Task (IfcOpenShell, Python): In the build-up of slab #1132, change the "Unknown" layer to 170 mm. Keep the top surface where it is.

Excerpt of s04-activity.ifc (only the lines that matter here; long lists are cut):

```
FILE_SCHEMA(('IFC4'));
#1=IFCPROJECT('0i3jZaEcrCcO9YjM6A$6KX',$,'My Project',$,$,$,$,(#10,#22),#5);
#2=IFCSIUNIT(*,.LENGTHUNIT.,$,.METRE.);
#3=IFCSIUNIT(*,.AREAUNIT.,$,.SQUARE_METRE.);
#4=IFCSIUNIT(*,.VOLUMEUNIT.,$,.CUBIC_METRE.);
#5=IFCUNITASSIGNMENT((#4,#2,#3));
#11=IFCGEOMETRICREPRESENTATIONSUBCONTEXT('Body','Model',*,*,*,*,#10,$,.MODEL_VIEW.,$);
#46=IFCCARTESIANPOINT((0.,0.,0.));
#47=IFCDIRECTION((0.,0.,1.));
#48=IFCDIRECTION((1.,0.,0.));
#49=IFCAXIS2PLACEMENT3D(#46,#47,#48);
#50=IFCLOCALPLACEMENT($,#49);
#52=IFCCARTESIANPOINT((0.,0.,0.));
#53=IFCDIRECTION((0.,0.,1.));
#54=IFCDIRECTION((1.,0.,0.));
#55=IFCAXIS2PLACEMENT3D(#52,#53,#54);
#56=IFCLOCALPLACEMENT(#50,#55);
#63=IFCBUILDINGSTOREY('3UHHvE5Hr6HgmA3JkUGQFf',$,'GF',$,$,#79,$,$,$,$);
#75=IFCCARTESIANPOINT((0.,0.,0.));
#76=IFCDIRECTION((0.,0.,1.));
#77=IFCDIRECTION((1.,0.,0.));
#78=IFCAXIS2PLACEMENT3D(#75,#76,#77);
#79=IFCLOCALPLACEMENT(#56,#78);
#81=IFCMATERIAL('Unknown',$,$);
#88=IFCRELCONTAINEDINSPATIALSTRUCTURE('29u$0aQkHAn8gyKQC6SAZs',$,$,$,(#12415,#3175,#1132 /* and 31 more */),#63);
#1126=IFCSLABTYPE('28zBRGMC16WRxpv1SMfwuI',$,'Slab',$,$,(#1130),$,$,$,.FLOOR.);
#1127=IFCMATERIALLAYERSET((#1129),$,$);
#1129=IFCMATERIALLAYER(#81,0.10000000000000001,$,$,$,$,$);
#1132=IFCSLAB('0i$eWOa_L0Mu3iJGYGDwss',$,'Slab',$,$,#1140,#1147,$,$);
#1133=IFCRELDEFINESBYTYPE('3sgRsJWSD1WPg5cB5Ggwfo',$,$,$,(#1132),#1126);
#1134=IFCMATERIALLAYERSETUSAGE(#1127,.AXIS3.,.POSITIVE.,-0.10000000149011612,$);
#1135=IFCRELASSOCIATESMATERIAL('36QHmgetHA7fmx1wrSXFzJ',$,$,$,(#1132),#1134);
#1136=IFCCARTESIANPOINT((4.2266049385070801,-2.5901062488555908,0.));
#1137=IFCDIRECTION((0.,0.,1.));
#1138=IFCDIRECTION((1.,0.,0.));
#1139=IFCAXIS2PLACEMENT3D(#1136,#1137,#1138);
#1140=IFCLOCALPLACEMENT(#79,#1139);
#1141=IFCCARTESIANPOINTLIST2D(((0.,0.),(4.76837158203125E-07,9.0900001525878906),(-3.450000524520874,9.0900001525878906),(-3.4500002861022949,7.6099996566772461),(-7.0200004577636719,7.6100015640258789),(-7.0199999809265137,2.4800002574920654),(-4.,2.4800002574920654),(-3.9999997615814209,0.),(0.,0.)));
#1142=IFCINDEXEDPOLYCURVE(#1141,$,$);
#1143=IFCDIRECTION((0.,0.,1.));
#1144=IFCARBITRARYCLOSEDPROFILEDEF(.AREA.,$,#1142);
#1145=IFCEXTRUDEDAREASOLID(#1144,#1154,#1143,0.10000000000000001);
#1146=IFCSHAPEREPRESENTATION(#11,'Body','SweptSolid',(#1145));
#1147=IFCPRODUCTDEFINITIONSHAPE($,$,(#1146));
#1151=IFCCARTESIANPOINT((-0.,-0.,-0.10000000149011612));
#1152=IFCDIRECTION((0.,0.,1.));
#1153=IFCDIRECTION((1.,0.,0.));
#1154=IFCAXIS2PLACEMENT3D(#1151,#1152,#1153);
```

```python
import ifcopenshell
import ifcopenshell.util.element
import ifcopenshell.util.representation
import ifcopenshell.util.unit

model = ifcopenshell.open("s04-activity.ifc")
unit_scale = ifcopenshell.util.unit.calculate_unit_scale(model)

layer_set = model.by_id(1127)
layer = next(l for l in layer_set.MaterialLayers if l.Material and l.Material.Name == "Unknown")
change = 0.17 / unit_scale - layer.LayerThickness
layer.LayerThickness += change

# Geometry does not follow the layer set by itself.
slabs = [e for e in ifcopenshell.util.element.get_elements_by_material(model, layer_set) if e.is_a("IfcSlab")]
for slab in sorted(slabs, key=lambda e: e.id()):
    body = ifcopenshell.util.representation.get_representation(slab, "Model", "Body")
    solid = body.Items[0]
    old_depth = solid.Depth
    solid.Depth += change
    # Extruded upwards: lower the start of the extrusion so the top stays.
    x, y, z = solid.Position.Location.Coordinates
    solid.Position.Location = model.createIfcCartesianPoint((x, y, z - change))
    print(slab.id(), f"{old_depth:g} -> {solid.Depth:g}")

# The layers are counted up from the underside, which has moved.
for usage in {ifcopenshell.util.element.get_material(slab) for slab in slabs}:
    usage.OffsetFromReferenceLine -= change

model.write("s04-activity_updated.ifc")
```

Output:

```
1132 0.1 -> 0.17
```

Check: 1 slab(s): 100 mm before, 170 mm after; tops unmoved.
